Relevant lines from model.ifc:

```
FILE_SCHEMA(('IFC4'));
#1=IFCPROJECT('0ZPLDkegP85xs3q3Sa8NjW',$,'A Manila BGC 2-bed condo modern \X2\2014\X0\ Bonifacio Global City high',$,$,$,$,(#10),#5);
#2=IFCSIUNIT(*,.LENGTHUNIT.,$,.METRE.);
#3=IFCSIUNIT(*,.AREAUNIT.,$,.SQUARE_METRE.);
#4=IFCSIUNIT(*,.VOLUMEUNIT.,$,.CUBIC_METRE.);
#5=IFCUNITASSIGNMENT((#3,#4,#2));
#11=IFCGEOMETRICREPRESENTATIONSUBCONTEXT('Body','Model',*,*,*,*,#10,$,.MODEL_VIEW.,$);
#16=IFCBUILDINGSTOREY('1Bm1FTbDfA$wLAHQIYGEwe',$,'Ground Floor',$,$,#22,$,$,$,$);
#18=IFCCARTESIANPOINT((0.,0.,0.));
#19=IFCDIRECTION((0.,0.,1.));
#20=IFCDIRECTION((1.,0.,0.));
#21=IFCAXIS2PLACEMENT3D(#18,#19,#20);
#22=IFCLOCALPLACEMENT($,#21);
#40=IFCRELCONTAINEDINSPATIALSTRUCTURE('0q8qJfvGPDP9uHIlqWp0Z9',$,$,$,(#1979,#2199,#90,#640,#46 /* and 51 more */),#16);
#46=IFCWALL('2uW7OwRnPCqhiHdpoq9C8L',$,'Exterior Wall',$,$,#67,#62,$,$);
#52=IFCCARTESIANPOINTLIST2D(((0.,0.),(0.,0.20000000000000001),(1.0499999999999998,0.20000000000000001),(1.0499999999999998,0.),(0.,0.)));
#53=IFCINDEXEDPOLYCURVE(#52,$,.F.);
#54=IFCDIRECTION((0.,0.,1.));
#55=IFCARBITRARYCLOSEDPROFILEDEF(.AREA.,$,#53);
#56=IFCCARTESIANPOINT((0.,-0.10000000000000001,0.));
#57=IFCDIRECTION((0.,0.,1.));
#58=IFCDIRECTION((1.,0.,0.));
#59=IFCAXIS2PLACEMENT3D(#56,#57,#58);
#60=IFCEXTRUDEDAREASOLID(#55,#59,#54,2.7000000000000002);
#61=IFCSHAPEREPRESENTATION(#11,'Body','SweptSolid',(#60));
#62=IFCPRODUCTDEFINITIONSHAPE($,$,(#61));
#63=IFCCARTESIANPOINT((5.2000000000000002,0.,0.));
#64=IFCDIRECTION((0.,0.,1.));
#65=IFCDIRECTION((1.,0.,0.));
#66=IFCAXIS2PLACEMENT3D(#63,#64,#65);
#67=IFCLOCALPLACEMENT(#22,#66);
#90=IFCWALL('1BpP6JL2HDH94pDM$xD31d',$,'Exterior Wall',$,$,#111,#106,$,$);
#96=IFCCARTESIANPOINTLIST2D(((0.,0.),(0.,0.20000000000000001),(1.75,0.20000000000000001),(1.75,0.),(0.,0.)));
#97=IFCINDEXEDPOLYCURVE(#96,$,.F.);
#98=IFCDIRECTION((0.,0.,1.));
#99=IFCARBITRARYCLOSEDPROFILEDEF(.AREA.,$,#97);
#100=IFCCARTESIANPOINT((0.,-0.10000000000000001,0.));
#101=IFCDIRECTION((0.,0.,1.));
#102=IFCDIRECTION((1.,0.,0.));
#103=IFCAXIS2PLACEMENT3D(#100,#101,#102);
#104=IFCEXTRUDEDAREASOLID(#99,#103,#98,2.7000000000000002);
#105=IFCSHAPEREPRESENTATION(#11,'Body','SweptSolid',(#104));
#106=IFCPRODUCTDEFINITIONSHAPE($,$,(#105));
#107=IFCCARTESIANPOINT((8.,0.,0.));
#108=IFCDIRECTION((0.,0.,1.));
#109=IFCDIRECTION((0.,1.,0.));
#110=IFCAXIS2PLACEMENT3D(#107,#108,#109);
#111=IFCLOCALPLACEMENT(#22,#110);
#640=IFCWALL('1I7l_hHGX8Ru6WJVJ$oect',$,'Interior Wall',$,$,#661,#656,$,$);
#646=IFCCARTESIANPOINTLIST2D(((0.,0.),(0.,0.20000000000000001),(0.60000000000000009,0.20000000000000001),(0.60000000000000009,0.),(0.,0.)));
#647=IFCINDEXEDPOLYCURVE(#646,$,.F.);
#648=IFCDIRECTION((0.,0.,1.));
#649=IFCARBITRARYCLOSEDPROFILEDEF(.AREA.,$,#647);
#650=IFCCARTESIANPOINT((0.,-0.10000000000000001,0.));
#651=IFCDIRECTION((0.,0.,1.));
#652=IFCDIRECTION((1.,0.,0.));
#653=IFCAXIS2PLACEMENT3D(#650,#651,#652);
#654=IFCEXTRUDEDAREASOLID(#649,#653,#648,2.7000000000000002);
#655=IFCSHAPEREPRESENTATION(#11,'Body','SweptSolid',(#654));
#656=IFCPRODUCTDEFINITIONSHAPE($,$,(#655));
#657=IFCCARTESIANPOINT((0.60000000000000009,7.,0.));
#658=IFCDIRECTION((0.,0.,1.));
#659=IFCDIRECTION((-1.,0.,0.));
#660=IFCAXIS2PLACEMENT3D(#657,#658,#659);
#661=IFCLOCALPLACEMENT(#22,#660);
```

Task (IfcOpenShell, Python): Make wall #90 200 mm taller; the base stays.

```python
import ifcopenshell
import ifcopenshell.geom
import ifcopenshell.util.representation
import ifcopenshell.util.shape
import ifcopenshell.util.unit

model = ifcopenshell.open("model.ifc")
unit_scale = ifcopenshell.util.unit.calculate_unit_scale(model)
settings = ifcopenshell.geom.settings()


def volume(element):
    """Net volume in cubic metres, openings subtracted."""
    shape = ifcopenshell.geom.create_shape(settings, element)
    return ifcopenshell.util.shape.get_volume(shape.geometry)


wall = model.by_guid("1BpP6JL2HDH94pDM$xD31d")
before = volume(wall)

body = ifcopenshell.util.representation.get_representation(wall, "Model", "Body")
solid = body.Items[0]
old_height = solid.Depth
solid.Depth += 0.2 / unit_scale
after = volume(wall)

print(f"height {old_height:g} -> {solid.Depth:g}, volume {before:.3f} -> {after:.3f} m3")

model.write("model_edited.ifc")
```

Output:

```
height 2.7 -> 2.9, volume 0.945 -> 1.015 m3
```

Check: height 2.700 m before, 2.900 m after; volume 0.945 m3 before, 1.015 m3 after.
